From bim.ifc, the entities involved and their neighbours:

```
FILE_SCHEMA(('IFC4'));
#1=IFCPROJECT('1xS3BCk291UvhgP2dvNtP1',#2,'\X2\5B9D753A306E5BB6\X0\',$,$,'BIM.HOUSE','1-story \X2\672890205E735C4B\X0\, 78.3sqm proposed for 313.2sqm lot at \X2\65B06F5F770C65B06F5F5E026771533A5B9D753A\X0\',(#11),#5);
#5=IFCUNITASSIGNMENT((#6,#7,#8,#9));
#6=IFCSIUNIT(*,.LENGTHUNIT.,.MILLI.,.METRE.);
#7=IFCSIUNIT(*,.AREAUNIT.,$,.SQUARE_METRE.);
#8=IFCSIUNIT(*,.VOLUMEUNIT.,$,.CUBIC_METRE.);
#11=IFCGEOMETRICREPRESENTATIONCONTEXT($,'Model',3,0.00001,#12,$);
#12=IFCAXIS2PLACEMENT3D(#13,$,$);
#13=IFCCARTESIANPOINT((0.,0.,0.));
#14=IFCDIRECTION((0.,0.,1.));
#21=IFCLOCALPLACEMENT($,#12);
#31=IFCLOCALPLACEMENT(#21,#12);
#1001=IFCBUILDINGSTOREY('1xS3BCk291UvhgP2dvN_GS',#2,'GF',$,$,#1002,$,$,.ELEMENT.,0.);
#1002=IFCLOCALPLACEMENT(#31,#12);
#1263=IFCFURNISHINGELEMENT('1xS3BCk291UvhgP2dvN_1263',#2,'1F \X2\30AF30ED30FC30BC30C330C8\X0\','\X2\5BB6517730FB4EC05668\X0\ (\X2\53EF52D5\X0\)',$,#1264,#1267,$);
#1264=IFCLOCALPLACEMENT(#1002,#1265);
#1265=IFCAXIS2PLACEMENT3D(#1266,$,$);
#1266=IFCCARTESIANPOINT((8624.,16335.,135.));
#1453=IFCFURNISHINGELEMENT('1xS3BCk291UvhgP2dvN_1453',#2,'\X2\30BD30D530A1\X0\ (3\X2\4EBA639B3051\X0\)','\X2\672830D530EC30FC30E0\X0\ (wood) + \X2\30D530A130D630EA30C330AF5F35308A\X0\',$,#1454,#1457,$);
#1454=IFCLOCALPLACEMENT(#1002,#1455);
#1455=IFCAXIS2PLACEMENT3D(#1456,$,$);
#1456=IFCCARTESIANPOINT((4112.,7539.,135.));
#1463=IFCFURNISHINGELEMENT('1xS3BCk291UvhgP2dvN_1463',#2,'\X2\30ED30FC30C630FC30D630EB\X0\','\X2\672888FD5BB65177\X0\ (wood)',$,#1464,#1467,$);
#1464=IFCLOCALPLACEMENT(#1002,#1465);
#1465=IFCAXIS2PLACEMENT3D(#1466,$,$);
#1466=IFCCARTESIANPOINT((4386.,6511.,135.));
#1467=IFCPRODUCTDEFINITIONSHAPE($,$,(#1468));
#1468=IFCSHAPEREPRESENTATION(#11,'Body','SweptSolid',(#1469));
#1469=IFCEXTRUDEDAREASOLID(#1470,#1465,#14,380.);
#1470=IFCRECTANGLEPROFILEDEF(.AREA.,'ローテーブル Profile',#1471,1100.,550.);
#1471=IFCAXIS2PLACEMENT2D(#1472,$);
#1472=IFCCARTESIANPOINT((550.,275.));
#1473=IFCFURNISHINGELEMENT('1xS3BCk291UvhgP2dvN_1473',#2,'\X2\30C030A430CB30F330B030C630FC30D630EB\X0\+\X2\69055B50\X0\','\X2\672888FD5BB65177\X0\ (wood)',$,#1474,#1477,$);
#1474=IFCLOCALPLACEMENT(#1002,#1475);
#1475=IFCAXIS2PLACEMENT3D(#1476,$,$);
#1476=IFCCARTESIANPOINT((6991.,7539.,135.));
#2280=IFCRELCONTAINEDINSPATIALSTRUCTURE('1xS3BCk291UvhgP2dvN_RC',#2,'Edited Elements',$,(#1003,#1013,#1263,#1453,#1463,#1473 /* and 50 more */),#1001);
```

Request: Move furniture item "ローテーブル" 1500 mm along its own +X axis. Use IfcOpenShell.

```python
import ifcopenshell
import ifcopenshell.api.geometry
import ifcopenshell.util.placement
import ifcopenshell.util.unit

model = ifcopenshell.open("bim.ifc")
unit_scale = ifcopenshell.util.unit.calculate_unit_scale(model)

item = model.by_id(1463)
matrix = ifcopenshell.util.placement.get_local_placement(item.ObjectPlacement)
matrix[:3, 3] += matrix[:3, 0] * 1.5 / unit_scale
ifcopenshell.api.geometry.edit_object_placement(model, product=item, matrix=matrix, is_si=False)

print(ifcopenshell.util.placement.get_local_placement(item.ObjectPlacement).round(3) + 0.0)

model.write("bim_rev.ifc")
```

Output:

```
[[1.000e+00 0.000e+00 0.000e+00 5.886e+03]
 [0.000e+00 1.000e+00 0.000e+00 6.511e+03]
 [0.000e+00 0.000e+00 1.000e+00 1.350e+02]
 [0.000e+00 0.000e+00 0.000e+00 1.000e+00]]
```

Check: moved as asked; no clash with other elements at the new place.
